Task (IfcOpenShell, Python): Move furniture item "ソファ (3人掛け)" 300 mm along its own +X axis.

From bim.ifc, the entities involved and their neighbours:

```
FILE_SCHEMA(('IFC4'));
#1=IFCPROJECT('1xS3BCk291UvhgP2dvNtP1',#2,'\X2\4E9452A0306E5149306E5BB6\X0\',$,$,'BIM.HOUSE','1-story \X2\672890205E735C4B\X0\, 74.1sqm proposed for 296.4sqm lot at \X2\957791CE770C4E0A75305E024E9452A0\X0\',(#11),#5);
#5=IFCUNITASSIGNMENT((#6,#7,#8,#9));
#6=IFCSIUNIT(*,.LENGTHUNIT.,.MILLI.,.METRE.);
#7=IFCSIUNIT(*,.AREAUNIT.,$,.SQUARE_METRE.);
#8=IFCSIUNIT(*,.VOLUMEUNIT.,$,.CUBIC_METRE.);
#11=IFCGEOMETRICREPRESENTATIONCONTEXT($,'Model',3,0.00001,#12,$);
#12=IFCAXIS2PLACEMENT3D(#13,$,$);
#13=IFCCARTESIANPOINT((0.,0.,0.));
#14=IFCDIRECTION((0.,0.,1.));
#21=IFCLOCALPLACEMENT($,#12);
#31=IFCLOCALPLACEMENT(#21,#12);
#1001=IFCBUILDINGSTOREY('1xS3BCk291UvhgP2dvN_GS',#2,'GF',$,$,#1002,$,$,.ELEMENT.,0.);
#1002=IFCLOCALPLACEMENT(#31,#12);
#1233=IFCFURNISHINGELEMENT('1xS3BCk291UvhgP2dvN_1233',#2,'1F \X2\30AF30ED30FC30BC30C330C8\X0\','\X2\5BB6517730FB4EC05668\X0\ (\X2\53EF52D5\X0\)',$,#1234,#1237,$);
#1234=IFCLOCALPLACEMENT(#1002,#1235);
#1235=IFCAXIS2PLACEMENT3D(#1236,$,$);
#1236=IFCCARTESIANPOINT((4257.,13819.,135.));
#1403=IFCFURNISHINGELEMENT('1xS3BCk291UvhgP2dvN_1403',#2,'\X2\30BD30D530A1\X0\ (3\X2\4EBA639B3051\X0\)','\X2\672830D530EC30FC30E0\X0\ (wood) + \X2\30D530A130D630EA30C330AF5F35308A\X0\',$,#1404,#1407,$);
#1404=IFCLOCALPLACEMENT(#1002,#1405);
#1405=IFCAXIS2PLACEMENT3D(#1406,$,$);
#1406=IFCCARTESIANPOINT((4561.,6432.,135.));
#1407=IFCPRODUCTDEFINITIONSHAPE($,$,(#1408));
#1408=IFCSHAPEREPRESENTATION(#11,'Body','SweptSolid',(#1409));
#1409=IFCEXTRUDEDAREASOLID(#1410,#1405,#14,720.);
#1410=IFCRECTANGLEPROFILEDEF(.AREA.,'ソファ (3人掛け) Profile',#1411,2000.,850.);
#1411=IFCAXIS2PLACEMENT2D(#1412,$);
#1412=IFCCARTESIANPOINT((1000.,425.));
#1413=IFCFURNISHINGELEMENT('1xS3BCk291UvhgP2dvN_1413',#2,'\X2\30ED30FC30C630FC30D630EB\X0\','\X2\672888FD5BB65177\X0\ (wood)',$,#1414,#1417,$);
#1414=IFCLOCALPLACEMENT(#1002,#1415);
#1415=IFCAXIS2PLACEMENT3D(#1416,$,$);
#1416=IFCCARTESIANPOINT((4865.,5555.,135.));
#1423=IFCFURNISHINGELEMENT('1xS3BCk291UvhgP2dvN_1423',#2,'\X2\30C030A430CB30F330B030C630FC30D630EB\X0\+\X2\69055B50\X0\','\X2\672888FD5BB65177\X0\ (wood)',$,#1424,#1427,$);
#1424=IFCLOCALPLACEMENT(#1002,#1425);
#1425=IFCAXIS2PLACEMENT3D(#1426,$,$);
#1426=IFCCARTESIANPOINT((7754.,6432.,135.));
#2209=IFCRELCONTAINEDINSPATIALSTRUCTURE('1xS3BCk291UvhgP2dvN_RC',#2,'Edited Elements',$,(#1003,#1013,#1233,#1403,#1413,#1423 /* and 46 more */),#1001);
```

```python
import ifcopenshell
import ifcopenshell.api.geometry
import ifcopenshell.util.placement
import ifcopenshell.util.unit

model = ifcopenshell.open("bim.ifc")
unit_scale = ifcopenshell.util.unit.calculate_unit_scale(model)

item = model.by_guid("1xS3BCk291UvhgP2dvN_1403")
matrix = ifcopenshell.util.placement.get_local_placement(item.ObjectPlacement)
matrix[:3, 3] += matrix[:3, 0] * 0.3 / unit_scale
ifcopenshell.api.geometry.edit_object_placement(model, product=item, matrix=matrix, is_si=False)

print(ifcopenshell.util.placement.get_local_placement(item.ObjectPlacement).round(3) + 0.0)

model.write("bim_updated.ifc")
```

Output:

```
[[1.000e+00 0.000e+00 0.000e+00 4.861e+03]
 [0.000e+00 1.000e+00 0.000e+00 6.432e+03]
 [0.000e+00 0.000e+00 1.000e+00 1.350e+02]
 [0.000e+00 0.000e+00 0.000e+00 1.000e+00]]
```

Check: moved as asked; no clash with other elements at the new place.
